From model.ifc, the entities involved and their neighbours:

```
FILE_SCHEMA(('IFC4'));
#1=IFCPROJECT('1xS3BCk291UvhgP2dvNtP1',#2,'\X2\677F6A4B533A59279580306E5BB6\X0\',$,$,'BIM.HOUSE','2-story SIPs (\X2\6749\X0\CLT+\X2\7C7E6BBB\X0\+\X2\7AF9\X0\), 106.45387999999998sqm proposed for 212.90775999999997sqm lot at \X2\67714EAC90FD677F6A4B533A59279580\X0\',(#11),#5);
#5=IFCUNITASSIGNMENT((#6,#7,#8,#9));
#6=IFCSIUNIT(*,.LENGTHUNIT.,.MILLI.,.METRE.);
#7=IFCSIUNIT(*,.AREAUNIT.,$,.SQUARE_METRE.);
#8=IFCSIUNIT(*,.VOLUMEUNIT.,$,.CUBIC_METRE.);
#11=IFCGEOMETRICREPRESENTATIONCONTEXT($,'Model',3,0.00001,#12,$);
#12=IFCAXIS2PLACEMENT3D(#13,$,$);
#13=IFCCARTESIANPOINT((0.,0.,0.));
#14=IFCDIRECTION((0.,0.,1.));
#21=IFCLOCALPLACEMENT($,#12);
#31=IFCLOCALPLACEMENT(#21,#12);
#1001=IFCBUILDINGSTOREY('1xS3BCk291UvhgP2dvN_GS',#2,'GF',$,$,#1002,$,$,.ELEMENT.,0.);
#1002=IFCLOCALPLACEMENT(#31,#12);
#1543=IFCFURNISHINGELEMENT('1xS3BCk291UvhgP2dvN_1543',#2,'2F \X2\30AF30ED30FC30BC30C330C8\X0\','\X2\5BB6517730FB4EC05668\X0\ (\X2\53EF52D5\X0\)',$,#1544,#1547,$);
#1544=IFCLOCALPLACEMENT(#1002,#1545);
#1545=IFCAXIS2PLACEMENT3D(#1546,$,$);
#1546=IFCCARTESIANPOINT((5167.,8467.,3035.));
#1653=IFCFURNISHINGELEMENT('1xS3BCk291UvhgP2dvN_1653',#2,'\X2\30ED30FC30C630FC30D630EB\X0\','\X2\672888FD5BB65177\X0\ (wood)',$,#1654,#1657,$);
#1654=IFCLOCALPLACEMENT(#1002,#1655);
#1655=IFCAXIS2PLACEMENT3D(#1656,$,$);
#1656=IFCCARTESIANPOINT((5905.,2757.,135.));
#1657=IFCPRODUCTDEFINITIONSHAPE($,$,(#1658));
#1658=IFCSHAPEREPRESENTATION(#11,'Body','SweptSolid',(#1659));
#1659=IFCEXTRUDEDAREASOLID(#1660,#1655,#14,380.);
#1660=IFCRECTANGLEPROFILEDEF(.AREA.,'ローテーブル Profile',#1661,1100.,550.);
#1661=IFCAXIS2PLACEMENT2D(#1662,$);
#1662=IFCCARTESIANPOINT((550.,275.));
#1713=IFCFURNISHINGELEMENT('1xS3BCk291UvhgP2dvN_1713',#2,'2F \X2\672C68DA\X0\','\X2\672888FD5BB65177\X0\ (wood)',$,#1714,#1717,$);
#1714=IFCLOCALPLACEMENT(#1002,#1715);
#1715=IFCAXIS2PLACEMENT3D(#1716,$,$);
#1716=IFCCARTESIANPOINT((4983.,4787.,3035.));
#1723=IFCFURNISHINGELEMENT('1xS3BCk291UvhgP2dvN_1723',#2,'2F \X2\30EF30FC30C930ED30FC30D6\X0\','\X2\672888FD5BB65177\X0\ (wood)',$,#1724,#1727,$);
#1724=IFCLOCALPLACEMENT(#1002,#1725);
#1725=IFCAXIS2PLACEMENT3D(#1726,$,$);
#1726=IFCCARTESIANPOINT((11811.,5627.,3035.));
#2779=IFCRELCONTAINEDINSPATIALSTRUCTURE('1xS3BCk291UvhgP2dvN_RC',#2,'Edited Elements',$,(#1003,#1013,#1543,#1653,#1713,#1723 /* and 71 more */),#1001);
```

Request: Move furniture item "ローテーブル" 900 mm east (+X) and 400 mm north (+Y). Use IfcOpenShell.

```python
import ifcopenshell
import ifcopenshell.api.geometry
import ifcopenshell.util.placement
import ifcopenshell.util.unit

model = ifcopenshell.open("model.ifc")
unit_scale = ifcopenshell.util.unit.calculate_unit_scale(model)

item = model.by_guid("1xS3BCk291UvhgP2dvN_1653")
matrix = ifcopenshell.util.placement.get_local_placement(item.ObjectPlacement)
matrix[0, 3] += 0.9 / unit_scale
matrix[1, 3] += 0.4 / unit_scale
ifcopenshell.api.geometry.edit_object_placement(model, product=item, matrix=matrix, is_si=False)

print(ifcopenshell.util.placement.get_local_placement(item.ObjectPlacement).round(3) + 0.0)

model.write("model_v2.ifc")
```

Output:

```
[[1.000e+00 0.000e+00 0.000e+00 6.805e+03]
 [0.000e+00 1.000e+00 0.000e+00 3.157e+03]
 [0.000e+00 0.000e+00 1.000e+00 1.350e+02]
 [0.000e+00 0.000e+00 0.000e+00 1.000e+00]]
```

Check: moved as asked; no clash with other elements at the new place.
